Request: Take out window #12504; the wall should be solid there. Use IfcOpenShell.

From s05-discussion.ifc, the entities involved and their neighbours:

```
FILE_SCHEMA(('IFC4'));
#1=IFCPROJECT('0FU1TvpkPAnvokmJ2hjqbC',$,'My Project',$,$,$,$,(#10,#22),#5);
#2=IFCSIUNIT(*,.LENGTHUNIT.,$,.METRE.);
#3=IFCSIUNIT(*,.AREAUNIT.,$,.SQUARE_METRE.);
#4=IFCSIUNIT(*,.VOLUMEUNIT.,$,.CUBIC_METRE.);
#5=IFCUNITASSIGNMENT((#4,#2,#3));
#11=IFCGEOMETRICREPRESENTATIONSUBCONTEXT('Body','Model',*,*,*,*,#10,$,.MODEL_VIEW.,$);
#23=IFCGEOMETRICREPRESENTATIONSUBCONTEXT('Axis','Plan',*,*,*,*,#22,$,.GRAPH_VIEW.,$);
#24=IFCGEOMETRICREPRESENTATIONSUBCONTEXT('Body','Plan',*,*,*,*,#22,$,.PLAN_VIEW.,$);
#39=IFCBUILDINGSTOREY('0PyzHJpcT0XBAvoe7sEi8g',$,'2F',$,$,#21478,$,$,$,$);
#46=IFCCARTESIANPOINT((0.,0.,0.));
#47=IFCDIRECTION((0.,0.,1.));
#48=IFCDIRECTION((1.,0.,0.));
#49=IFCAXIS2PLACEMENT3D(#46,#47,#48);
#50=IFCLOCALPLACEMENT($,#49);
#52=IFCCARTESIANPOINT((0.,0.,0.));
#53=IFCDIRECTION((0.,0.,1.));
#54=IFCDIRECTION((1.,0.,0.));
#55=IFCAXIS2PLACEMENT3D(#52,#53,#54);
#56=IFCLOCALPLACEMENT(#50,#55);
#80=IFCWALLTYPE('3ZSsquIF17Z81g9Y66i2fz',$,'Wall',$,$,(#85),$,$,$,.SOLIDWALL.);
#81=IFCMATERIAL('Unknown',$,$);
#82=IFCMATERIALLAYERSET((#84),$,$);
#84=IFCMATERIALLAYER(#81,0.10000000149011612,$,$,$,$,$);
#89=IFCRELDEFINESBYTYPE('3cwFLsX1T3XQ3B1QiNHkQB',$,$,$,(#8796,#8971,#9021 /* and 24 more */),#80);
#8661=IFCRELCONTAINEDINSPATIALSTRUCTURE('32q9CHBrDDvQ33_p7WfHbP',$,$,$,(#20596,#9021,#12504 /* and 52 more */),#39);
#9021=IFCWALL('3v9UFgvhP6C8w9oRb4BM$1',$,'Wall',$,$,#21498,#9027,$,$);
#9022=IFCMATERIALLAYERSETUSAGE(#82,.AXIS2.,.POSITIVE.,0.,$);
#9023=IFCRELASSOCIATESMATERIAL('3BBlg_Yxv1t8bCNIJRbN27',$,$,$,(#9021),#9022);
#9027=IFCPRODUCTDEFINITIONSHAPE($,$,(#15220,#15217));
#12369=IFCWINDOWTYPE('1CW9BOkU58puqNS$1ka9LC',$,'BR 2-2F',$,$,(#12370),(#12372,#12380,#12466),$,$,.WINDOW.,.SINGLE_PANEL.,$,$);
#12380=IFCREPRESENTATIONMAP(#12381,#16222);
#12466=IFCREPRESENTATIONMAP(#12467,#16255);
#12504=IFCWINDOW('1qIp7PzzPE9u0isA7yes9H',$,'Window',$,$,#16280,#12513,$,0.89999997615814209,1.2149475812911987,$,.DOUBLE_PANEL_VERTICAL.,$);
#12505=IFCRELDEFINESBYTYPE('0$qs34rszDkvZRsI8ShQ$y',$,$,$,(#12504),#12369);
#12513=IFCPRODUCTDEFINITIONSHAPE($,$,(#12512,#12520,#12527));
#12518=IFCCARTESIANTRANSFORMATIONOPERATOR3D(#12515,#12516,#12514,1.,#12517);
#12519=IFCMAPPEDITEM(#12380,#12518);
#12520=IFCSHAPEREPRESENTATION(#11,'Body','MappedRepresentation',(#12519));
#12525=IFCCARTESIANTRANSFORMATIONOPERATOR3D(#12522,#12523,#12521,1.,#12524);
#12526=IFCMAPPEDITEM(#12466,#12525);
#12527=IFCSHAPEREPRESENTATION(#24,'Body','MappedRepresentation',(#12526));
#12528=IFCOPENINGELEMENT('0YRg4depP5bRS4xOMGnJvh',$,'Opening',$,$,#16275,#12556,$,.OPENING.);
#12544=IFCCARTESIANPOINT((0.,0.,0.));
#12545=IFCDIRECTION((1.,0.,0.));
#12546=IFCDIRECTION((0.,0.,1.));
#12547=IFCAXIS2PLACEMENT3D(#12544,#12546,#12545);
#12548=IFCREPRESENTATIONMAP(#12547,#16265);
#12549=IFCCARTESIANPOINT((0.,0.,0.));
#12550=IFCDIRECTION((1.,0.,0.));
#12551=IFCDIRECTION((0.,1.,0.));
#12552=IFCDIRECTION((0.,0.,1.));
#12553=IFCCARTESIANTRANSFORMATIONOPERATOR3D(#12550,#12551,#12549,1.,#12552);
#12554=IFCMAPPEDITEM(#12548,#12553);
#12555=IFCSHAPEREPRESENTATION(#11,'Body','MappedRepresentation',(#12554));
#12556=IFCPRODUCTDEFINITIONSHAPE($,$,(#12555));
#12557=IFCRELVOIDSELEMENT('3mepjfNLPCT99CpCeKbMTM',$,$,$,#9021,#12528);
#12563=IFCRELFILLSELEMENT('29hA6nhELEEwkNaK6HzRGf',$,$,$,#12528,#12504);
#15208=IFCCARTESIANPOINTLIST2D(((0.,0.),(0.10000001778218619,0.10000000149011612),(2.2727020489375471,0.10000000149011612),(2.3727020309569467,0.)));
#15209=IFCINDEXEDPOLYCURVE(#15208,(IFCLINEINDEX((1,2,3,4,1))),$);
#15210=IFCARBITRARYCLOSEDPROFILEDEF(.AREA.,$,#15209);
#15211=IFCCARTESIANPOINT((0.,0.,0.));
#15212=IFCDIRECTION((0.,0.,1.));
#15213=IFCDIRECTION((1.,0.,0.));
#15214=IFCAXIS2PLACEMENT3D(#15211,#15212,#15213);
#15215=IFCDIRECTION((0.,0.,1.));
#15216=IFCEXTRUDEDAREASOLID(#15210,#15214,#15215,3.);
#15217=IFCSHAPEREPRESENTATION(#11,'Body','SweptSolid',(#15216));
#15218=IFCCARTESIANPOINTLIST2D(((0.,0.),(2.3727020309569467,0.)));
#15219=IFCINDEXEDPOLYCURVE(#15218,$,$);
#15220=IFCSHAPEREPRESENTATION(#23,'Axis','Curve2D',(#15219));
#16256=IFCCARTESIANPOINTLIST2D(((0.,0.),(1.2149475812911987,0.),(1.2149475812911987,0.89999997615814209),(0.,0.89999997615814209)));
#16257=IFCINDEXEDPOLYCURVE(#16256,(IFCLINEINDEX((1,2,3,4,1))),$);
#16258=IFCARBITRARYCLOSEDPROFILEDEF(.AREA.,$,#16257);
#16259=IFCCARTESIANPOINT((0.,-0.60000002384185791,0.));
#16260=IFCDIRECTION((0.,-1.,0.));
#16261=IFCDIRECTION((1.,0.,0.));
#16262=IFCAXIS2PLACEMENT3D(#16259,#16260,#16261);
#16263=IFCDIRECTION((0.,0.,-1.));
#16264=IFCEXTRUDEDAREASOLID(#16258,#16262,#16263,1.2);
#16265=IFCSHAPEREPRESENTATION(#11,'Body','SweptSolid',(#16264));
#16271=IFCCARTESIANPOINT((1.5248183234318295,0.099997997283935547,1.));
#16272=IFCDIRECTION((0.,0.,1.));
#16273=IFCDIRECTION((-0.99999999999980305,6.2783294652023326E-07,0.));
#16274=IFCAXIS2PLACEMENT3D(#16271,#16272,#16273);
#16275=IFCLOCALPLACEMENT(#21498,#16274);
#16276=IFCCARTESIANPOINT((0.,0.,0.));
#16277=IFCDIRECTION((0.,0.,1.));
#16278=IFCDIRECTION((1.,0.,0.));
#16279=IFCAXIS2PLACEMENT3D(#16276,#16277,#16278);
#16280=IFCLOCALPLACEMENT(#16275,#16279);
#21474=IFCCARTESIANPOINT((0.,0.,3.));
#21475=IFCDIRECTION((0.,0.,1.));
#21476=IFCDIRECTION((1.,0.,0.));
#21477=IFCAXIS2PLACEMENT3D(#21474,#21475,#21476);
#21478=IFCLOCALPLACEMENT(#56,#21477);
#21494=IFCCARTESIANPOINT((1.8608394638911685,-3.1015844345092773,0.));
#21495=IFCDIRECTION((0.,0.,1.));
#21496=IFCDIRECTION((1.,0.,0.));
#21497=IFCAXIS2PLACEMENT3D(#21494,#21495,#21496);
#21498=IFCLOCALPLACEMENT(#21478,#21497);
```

```python
import ifcopenshell
import ifcopenshell.api.feature
import ifcopenshell.api.root
import ifcopenshell.geom
import ifcopenshell.util.shape

model = ifcopenshell.open("s05-discussion.ifc")
settings = ifcopenshell.geom.settings()


def volume(element):
    """Net volume in cubic metres, openings subtracted."""
    shape = ifcopenshell.geom.create_shape(settings, element)
    return ifcopenshell.util.shape.get_volume(shape.geometry)


window = model.by_guid("1qIp7PzzPE9u0isA7yes9H")
opening = window.FillsVoids[0].RelatingOpeningElement
wall = opening.VoidsElements[0].RelatingBuildingElement
before = volume(wall)

ifcopenshell.api.root.remove_product(model, product=window)
ifcopenshell.api.feature.remove_feature(model, feature=opening)

after = volume(wall)

print(f"wall volume {before:.3f} -> {after:.3f} m3")

model.write("s05-discussion_v2.ifc")
```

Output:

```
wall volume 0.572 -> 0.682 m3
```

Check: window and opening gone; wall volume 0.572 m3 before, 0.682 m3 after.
